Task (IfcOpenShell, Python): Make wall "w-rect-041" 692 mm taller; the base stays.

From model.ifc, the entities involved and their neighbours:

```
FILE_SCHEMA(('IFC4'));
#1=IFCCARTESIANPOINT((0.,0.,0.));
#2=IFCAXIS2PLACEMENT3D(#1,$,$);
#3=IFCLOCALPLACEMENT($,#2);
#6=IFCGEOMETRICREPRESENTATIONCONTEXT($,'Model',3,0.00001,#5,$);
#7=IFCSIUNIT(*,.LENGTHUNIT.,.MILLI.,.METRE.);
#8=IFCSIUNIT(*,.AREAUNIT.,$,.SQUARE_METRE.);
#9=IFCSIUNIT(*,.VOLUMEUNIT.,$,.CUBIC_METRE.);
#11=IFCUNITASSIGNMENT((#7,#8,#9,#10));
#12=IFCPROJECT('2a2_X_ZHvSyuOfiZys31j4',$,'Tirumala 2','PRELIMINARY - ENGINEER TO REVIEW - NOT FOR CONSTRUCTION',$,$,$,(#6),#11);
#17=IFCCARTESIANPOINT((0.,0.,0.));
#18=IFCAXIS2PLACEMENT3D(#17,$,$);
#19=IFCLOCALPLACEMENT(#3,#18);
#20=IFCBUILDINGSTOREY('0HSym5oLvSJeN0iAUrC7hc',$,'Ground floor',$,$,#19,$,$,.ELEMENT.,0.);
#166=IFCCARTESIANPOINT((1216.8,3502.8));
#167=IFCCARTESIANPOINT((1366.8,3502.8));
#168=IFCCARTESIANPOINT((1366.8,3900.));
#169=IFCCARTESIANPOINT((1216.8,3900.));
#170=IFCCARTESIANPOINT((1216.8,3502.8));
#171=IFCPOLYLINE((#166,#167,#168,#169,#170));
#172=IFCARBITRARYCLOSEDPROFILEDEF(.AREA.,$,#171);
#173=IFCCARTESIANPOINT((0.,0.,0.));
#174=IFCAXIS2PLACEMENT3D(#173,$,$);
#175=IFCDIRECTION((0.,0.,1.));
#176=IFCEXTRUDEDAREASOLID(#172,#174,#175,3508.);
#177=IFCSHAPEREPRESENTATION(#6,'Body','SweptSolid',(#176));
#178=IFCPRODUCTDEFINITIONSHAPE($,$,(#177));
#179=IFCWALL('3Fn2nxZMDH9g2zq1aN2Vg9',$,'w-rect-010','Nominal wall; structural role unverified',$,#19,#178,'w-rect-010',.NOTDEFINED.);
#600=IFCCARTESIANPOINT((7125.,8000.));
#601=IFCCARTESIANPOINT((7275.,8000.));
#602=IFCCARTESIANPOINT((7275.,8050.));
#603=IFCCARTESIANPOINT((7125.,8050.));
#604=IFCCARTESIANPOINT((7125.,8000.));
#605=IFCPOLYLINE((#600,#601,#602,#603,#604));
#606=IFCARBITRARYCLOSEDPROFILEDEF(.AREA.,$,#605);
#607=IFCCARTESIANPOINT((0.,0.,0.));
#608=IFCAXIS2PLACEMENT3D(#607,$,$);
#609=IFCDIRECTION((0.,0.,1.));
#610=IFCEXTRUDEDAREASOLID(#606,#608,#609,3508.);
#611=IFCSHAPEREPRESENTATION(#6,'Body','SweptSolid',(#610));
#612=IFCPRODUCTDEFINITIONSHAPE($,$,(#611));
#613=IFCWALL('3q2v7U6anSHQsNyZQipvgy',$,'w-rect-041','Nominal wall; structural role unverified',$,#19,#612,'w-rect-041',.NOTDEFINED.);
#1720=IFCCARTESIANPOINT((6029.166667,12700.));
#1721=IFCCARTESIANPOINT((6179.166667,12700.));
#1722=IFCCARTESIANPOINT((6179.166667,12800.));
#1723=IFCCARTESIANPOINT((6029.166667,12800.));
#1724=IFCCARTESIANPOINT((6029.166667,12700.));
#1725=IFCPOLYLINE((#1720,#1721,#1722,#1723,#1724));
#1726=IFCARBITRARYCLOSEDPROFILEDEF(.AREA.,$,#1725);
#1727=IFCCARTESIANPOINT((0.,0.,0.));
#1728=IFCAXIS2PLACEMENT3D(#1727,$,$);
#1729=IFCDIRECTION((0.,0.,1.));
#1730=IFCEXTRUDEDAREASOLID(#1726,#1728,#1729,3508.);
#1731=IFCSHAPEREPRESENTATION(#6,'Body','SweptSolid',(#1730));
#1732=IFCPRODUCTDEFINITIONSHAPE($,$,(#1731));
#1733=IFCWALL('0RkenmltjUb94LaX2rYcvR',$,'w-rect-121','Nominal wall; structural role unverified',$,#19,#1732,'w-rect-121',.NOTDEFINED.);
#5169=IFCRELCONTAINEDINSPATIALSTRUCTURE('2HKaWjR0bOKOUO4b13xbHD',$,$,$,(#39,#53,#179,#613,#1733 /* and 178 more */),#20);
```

```python
import ifcopenshell
import ifcopenshell.geom
import ifcopenshell.util.shape
import ifcopenshell.util.unit

model = ifcopenshell.open("model.ifc")
unit_scale = ifcopenshell.util.unit.calculate_unit_scale(model)
settings = ifcopenshell.geom.settings()


def volume(element):
    """Net volume in cubic metres, openings subtracted."""
    shape = ifcopenshell.geom.create_shape(settings, element)
    return ifcopenshell.util.shape.get_volume(shape.geometry)


wall = model.by_guid("3q2v7U6anSHQsNyZQipvgy")
before = volume(wall)

body = next(r for r in wall.Representation.Representations if r.RepresentationIdentifier == "Body")
solid = body.Items[0]
old_height = solid.Depth
solid.Depth += 0.692 / unit_scale
after = volume(wall)

print(f"height {old_height:g} -> {solid.Depth:g}, volume {before:.3f} -> {after:.3f} m3")

model.write("model_updated.ifc")
```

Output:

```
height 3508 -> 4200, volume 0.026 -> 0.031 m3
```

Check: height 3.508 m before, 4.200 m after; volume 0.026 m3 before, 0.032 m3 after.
